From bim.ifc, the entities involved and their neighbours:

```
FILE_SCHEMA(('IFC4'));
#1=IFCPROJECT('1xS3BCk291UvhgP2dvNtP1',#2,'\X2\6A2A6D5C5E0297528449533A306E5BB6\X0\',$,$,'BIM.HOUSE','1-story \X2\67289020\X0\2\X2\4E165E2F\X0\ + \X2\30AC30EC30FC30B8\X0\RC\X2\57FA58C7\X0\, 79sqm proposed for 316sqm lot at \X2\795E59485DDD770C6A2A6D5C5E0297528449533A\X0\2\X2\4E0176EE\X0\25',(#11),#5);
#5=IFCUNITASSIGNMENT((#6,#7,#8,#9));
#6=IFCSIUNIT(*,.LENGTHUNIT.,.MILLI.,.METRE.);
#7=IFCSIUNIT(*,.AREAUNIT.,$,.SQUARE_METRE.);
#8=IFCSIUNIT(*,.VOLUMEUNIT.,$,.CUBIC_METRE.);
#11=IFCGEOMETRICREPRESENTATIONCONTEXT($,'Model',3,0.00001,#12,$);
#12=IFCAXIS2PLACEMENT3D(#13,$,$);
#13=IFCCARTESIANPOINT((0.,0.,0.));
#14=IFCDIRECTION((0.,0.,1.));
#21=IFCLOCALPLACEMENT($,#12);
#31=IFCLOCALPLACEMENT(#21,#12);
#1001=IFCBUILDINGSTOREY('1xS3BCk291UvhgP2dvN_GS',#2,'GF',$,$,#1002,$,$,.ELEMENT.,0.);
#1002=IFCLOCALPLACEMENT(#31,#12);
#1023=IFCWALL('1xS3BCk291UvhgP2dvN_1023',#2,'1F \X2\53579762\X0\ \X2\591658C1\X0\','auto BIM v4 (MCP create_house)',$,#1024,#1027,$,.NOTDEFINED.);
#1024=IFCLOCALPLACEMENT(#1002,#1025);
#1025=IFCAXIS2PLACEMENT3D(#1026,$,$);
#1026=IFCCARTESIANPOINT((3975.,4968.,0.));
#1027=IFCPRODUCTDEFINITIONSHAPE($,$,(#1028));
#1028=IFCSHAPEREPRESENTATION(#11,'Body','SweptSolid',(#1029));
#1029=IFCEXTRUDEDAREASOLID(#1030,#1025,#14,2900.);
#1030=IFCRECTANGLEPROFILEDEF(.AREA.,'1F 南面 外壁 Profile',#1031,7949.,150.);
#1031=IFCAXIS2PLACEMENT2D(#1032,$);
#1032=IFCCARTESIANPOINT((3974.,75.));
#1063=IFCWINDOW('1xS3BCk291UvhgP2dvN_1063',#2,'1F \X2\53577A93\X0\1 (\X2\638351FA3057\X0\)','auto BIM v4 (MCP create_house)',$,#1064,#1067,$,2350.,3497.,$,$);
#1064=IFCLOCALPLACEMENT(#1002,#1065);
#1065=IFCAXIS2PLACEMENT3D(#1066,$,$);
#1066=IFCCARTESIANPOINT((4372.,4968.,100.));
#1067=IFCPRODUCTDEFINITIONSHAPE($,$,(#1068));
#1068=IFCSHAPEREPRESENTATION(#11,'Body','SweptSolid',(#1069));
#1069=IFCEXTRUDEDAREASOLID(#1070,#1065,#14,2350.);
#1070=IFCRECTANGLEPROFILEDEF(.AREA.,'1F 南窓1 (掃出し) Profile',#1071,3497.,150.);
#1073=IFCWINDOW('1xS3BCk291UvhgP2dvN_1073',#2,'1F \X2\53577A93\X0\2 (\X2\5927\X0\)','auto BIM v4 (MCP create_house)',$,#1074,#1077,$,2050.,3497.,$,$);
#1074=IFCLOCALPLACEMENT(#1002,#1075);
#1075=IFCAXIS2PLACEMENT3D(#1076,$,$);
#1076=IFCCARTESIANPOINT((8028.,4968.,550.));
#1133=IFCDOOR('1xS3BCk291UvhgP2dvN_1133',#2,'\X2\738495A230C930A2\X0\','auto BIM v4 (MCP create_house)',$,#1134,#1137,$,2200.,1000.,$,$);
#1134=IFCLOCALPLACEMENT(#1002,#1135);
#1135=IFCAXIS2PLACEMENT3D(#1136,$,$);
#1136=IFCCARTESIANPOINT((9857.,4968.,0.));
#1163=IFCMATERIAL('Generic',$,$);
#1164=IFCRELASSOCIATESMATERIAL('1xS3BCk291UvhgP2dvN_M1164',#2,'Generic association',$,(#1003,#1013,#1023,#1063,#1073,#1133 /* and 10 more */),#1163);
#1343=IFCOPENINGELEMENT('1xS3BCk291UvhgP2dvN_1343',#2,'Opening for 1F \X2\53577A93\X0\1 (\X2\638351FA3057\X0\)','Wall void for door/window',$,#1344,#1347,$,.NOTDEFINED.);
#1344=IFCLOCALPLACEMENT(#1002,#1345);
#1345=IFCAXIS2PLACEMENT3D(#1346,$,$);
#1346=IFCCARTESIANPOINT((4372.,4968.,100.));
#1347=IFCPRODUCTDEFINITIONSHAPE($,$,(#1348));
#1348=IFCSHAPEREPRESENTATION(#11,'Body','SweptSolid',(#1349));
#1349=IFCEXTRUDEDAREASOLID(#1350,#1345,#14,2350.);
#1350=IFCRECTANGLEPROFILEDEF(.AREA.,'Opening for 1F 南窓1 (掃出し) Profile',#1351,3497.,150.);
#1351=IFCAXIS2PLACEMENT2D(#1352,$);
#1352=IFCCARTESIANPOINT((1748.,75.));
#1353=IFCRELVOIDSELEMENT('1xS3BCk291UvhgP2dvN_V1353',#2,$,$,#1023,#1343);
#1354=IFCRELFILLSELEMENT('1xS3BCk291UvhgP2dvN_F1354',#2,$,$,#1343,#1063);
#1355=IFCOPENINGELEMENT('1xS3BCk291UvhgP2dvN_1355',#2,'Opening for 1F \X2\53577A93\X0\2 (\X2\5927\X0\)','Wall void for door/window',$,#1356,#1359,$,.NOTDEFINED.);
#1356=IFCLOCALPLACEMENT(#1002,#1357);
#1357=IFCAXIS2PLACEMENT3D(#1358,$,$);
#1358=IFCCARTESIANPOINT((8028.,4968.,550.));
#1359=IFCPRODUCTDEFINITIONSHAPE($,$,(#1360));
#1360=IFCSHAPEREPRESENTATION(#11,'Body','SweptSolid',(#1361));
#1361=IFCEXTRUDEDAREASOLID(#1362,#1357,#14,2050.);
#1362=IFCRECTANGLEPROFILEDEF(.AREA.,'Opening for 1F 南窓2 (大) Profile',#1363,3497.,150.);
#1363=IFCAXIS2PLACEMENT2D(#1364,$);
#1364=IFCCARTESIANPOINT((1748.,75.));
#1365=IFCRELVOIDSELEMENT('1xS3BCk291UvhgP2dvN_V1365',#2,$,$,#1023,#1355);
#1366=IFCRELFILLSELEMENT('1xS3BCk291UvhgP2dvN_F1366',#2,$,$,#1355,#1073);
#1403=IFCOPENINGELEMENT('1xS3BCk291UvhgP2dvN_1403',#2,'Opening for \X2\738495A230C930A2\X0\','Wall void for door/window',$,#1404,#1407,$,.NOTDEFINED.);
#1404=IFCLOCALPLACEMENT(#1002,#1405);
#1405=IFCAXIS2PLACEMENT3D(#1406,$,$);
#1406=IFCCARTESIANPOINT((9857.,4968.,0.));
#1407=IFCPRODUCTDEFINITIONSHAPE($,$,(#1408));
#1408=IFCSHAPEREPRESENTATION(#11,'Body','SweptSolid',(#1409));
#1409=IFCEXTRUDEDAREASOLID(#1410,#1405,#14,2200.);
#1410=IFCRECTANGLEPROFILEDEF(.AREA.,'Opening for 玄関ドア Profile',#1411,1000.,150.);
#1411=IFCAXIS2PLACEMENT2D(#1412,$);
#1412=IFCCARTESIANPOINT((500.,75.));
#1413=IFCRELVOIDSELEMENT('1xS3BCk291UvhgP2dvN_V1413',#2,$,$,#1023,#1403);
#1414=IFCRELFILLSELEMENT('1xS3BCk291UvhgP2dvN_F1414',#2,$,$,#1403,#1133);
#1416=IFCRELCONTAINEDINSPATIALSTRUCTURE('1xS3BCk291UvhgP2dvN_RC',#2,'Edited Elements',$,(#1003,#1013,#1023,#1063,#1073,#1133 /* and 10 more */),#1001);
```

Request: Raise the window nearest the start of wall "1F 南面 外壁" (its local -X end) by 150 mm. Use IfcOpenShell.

```python
import numpy as np
import ifcopenshell
import ifcopenshell.api.geometry
import ifcopenshell.util.placement
import ifcopenshell.util.unit

model = ifcopenshell.open("bim.ifc")
unit_scale = ifcopenshell.util.unit.calculate_unit_scale(model)

window = model.by_id(1063)
opening = window.FillsVoids[0].RelatingOpeningElement
dz = 0.15 / unit_scale

shift = np.array([0.0, 0.0, dz])
# The window is not placed relative to its opening, so move both.
for product in (opening, window):
    matrix = ifcopenshell.util.placement.get_local_placement(product.ObjectPlacement)
    matrix[:3, 3] += shift
    ifcopenshell.api.geometry.edit_object_placement(model, product=product, matrix=matrix, is_si=False)

print(f"moved by {dz * unit_scale:+.3f} m")

model.write("bim_updated.ifc")
```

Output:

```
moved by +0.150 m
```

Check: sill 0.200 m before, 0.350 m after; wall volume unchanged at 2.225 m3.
